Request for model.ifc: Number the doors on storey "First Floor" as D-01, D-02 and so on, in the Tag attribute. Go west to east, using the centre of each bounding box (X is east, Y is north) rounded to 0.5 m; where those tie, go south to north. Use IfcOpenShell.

First a look at what the model holds.

```python
import ifcopenshell
import ifcopenshell.util.element
import ifcopenshell.util.placement

model = ifcopenshell.open("model.ifc")
print(model.schema)
storey = next(s for s in model.by_type("IfcBuildingStorey") if s.Name == "First Floor")
doors = [e for e in ifcopenshell.util.element.get_decomposition(storey) if e.is_a("IfcDoor")]
for e in sorted(doors, key=lambda e: e.id()):
    origin = ifcopenshell.util.placement.get_local_placement(e.ObjectPlacement)[:3, 3]
    print(e.id(), e.Tag, e.Name, origin.round(2) + 0.0, sep=" | ")
```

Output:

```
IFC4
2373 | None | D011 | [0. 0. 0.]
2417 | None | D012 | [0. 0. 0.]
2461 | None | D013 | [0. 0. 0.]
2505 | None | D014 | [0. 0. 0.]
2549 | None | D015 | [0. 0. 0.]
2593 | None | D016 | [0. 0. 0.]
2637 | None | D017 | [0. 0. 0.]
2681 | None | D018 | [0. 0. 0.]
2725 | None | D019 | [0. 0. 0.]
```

```python
import ifcopenshell
import ifcopenshell.geom
import ifcopenshell.util.element
import ifcopenshell.util.shape

model = ifcopenshell.open("model.ifc")
settings = ifcopenshell.geom.settings()
settings.set("use-world-coords", True)


def centre(element):
    shape = ifcopenshell.geom.create_shape(settings, element)
    return ifcopenshell.util.shape.get_bbox_centroid(shape.geometry)


storey = next(s for s in model.by_type("IfcBuildingStorey") if s.Name == "First Floor")
doors = [e for e in ifcopenshell.util.element.get_decomposition(storey) if e.is_a("IfcDoor")]

# Insertion points can sit at a corner or the storey origin, so sort by the geometry (in metres).
centres = {e: centre(e) for e in doors}
doors.sort(key=lambda e: (round(centres[e][0] / 0.5), centres[e][1]))

for i, e in enumerate(doors, start=1):
    number = f"D-{i:02d}"
    e.Tag = number
    print(e.id(), number)

model.write("model_rev.ifc")
```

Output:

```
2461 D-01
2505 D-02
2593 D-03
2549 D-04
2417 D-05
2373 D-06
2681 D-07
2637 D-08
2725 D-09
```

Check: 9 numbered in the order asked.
